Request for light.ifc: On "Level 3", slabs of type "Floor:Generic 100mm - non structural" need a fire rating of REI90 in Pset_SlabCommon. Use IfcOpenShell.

First a look at what the model holds.

```python
import ifcopenshell
import ifcopenshell.util.element

model = ifcopenshell.open("light.ifc")
print(model.schema)
storey = next(s for s in model.by_type("IfcBuildingStorey") if s.Name == "Level 3")
slabs = [e for e in ifcopenshell.util.element.get_decomposition(storey) if e.is_a("IfcSlab")]
seen = {}
for e in slabs:
    element_type = ifcopenshell.util.element.get_type(e)
    key = (element_type.Name if element_type != e and element_type else None, ifcopenshell.util.element.get_pset(e, "Pset_SlabCommon", "FireRating"))
    seen[key] = seen.get(key, 0) + 1
for (name, value), count in sorted(seen.items(), key=str):
    print(count, "x", name, "|", value)
```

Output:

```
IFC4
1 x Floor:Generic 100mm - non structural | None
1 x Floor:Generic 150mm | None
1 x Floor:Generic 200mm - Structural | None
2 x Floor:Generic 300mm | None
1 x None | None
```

```python
import ifcopenshell
import ifcopenshell.api.pset
import ifcopenshell.util.element

model = ifcopenshell.open("light.ifc")

storey = next(s for s in model.by_type("IfcBuildingStorey") if s.Name == "Level 3")
slabs = [e for e in ifcopenshell.util.element.get_decomposition(storey) if e.is_a("IfcSlab")]

count = 0
for e in slabs:
    element_type = ifcopenshell.util.element.get_type(e)
    if element_type in (None, e) or element_type.Name != "Floor:Generic 100mm - non structural":
        continue
    # add_pset returns the element's existing set when there is one.
    pset = ifcopenshell.api.pset.add_pset(model, product=e, name="Pset_SlabCommon")
    ifcopenshell.api.pset.edit_pset(model, pset=pset, properties={"FireRating": "REI90"})
    count += 1

print(count, "slabs updated")

model.write("light_v2.ifc")
```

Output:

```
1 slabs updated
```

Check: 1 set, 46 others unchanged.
